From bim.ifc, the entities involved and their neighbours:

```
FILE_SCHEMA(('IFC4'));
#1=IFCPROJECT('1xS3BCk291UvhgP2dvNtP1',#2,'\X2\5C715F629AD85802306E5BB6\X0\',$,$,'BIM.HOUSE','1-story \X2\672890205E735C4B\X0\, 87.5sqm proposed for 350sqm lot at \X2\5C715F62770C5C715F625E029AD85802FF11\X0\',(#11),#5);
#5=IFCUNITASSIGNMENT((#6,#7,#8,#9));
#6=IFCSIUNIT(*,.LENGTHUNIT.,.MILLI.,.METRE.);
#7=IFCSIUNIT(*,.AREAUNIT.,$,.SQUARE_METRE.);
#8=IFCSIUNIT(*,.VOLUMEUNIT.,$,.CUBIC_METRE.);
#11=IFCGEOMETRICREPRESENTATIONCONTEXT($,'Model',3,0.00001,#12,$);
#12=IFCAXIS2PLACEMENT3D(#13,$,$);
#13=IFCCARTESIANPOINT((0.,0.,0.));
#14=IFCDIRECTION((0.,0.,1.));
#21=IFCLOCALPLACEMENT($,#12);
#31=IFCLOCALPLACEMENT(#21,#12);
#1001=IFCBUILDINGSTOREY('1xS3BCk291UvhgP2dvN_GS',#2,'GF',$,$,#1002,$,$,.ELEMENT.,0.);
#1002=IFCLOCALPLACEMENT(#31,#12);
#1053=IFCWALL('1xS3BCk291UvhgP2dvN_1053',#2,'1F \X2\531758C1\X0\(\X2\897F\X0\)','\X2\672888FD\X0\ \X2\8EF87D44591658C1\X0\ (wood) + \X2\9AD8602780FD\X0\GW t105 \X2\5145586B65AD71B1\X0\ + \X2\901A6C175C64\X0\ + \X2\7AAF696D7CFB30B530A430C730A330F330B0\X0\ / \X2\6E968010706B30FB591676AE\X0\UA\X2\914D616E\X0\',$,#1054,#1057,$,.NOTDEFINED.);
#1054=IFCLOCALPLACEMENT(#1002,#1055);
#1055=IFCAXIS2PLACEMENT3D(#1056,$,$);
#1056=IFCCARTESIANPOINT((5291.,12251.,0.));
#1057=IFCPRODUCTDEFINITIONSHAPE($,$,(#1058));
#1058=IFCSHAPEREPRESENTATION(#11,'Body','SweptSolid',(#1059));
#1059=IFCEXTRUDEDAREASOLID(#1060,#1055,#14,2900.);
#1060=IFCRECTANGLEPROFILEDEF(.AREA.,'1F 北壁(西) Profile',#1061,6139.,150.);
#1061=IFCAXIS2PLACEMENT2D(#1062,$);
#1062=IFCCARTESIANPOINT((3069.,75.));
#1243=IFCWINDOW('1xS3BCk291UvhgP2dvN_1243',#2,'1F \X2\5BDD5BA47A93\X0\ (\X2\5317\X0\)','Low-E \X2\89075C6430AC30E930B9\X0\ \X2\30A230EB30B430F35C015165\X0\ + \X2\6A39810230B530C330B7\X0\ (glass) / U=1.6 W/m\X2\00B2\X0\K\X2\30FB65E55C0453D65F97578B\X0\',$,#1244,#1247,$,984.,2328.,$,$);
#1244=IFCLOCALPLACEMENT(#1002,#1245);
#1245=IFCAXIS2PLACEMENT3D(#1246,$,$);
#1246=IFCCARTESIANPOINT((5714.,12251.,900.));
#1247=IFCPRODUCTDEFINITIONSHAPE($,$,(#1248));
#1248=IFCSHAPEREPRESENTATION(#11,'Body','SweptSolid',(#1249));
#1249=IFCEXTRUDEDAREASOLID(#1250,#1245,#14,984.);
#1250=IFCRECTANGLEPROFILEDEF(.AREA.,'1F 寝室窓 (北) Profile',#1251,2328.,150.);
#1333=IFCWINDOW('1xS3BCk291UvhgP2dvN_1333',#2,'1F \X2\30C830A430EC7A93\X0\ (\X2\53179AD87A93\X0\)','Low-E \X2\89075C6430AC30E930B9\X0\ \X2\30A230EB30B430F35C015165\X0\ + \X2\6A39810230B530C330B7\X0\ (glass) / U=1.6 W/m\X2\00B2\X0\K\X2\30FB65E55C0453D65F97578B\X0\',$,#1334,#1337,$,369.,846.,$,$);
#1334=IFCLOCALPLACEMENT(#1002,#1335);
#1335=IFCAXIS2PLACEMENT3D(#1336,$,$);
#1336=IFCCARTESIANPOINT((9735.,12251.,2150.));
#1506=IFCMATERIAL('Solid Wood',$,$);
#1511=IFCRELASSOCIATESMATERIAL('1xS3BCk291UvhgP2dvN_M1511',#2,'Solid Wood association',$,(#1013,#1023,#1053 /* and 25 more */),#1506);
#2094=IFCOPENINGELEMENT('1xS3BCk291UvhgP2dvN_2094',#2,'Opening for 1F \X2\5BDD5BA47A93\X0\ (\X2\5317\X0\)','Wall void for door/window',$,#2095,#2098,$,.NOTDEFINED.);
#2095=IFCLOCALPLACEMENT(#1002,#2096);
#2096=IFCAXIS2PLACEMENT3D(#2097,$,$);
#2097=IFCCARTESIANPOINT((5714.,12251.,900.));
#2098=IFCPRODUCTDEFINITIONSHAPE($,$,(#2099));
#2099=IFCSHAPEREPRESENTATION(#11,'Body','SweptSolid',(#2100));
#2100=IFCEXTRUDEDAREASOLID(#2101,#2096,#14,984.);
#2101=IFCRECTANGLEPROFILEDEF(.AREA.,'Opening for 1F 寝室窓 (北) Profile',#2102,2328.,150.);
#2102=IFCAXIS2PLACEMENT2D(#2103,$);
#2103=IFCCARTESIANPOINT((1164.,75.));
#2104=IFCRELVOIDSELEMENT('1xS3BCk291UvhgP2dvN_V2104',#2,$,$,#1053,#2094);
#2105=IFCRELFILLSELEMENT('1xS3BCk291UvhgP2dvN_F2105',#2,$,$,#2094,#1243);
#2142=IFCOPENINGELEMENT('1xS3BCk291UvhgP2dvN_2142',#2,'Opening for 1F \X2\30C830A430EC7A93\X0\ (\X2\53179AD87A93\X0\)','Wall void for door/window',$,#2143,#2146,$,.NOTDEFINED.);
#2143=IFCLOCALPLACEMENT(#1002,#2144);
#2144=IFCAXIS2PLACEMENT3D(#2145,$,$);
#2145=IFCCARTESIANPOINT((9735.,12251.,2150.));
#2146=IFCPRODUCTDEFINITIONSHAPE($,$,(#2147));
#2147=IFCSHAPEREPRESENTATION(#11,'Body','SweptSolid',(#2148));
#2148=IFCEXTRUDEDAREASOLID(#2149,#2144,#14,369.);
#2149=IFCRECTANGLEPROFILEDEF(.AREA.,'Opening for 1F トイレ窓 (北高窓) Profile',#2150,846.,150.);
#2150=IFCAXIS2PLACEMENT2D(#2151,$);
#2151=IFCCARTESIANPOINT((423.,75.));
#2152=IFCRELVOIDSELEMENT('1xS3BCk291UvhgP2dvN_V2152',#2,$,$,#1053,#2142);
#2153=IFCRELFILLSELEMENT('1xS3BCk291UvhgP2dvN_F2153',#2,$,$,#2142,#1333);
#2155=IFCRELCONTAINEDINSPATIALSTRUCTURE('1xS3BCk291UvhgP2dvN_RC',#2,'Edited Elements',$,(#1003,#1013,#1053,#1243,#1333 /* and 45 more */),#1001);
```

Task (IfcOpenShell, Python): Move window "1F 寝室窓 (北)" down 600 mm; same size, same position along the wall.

```python
import numpy as np
import ifcopenshell
import ifcopenshell.api.geometry
import ifcopenshell.util.placement
import ifcopenshell.util.unit

model = ifcopenshell.open("bim.ifc")
unit_scale = ifcopenshell.util.unit.calculate_unit_scale(model)

window = model.by_guid("1xS3BCk291UvhgP2dvN_1243")
opening = window.FillsVoids[0].RelatingOpeningElement
dz = -0.6 / unit_scale

shift = np.array([0.0, 0.0, dz])
# The window is not placed relative to its opening, so move both.
for product in (opening, window):
    matrix = ifcopenshell.util.placement.get_local_placement(product.ObjectPlacement)
    matrix[:3, 3] += shift
    ifcopenshell.api.geometry.edit_object_placement(model, product=product, matrix=matrix, is_si=False)

print(f"moved by {dz * unit_scale:+.3f} m")

model.write("bim_rev.ifc")
```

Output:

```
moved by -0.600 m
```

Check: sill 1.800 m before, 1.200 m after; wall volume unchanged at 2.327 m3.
